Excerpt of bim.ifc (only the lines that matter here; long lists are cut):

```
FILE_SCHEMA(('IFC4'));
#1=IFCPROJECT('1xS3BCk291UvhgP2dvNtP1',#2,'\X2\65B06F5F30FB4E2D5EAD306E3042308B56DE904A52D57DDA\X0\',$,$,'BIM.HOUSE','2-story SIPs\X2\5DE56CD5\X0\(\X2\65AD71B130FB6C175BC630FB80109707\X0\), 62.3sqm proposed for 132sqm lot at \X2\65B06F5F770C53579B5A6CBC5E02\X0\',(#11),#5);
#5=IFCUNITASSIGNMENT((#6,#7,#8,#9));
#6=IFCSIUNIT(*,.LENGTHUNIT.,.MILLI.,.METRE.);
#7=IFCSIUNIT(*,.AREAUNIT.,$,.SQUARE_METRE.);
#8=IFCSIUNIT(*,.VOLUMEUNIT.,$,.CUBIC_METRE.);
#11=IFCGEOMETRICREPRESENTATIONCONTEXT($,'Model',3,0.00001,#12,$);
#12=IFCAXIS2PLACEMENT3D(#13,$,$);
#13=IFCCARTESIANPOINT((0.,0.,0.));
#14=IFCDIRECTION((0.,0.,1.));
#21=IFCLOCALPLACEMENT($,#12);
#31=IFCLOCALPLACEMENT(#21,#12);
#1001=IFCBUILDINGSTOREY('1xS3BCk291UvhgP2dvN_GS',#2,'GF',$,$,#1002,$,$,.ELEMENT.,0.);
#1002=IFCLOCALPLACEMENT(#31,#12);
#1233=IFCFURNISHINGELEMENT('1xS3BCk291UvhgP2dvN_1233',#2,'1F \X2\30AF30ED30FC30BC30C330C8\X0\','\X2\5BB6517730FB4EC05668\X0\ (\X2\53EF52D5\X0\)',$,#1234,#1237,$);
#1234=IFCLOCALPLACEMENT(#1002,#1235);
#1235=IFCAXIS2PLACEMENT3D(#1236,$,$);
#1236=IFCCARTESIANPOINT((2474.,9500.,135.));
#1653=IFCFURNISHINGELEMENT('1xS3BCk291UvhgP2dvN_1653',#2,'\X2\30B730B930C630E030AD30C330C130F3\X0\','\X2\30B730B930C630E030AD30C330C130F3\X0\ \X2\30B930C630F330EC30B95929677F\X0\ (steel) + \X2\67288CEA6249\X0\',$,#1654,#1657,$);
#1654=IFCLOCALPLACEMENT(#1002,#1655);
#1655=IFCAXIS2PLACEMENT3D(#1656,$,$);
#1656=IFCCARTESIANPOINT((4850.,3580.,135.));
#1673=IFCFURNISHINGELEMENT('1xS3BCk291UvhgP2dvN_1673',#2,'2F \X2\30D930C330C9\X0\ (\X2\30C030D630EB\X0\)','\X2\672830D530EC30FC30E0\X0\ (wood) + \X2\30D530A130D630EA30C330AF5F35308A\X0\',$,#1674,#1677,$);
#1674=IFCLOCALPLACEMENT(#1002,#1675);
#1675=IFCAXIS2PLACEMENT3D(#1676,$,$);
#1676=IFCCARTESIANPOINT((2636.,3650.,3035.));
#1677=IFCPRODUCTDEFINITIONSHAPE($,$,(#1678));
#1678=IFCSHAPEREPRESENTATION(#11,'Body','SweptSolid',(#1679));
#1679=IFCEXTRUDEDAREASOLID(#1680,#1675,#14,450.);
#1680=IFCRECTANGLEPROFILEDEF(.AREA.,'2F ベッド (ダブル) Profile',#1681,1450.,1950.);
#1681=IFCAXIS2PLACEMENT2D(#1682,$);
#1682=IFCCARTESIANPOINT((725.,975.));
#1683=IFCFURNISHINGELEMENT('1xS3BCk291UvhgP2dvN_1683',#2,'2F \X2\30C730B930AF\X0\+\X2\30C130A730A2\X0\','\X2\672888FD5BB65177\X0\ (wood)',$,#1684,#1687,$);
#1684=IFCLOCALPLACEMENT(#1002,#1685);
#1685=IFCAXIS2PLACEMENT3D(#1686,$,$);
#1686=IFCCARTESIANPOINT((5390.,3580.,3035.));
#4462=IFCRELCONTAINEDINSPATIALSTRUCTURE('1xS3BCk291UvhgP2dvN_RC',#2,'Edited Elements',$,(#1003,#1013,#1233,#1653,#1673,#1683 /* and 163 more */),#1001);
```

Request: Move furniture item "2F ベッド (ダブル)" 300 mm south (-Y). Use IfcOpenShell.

```python
import ifcopenshell
import ifcopenshell.api.geometry
import ifcopenshell.util.placement

model = ifcopenshell.open("bim.ifc")

item = model.by_guid("1xS3BCk291UvhgP2dvN_1673")
matrix = ifcopenshell.util.placement.get_local_placement(item.ObjectPlacement)
matrix[1, 3] -= 300.0
ifcopenshell.api.geometry.edit_object_placement(model, product=item, matrix=matrix, is_si=False)

print(ifcopenshell.util.placement.get_local_placement(item.ObjectPlacement).round(3) + 0.0)

model.write("bim-out.ifc")
```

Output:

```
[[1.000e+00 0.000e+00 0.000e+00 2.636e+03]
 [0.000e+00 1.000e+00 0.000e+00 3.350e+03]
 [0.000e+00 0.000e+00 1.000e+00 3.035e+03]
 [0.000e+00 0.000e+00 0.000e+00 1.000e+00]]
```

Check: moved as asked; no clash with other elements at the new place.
